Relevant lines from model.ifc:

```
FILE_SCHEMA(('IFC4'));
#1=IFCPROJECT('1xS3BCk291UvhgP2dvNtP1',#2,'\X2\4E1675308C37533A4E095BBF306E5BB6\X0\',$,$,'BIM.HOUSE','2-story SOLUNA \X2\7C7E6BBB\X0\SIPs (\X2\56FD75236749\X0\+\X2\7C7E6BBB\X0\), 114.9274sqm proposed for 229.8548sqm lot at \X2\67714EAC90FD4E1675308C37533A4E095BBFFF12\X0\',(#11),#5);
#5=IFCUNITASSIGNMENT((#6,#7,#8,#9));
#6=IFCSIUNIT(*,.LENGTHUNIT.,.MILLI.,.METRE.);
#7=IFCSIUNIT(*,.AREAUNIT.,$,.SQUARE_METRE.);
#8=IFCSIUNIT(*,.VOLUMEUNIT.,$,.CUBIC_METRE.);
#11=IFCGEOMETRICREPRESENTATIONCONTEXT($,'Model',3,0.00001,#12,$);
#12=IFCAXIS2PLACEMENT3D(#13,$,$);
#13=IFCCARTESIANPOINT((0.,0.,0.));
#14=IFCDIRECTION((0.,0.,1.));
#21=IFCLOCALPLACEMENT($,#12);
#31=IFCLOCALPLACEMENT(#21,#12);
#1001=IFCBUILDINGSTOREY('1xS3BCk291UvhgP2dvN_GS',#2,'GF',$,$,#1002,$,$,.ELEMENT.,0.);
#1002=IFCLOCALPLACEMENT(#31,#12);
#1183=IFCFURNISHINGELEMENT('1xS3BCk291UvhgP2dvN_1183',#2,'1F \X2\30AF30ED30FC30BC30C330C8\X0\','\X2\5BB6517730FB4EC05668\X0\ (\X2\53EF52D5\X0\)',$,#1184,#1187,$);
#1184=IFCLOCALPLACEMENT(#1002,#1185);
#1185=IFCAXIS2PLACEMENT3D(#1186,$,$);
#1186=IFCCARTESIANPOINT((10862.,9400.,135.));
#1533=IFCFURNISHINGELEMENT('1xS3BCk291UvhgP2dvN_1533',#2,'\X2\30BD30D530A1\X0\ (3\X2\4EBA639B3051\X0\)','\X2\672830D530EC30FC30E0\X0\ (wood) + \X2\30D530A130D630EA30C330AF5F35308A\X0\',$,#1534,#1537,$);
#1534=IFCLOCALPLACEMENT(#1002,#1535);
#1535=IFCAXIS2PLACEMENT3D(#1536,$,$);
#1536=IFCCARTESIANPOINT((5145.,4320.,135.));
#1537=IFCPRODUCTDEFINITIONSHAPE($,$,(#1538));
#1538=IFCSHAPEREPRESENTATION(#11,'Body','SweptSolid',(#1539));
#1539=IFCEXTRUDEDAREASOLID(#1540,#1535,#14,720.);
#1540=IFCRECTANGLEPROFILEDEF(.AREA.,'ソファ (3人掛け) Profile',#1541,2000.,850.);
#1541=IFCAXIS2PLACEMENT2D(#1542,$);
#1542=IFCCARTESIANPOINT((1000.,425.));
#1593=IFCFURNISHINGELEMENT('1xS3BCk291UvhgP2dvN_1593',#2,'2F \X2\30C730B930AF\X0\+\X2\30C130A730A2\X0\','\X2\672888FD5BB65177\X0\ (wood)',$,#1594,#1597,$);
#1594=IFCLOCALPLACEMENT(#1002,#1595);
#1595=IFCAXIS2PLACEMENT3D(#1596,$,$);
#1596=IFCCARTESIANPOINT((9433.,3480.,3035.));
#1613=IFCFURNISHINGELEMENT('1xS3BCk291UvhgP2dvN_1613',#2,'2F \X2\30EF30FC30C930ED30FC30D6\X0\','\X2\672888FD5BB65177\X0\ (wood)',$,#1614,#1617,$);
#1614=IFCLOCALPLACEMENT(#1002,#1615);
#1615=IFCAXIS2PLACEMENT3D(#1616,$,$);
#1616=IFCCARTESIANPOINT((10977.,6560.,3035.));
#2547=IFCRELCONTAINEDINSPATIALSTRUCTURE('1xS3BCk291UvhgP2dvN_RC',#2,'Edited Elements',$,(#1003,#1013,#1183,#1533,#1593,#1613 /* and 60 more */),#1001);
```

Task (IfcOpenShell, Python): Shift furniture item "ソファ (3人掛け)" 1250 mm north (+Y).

```python
import ifcopenshell
import ifcopenshell.api.geometry
import ifcopenshell.util.placement

model = ifcopenshell.open("model.ifc")

item = model.by_guid("1xS3BCk291UvhgP2dvN_1533")
matrix = ifcopenshell.util.placement.get_local_placement(item.ObjectPlacement)
matrix[1, 3] += 1250.0
ifcopenshell.api.geometry.edit_object_placement(model, product=item, matrix=matrix, is_si=False)

print(ifcopenshell.util.placement.get_local_placement(item.ObjectPlacement).round(3) + 0.0)

model.write("model_edited.ifc")
```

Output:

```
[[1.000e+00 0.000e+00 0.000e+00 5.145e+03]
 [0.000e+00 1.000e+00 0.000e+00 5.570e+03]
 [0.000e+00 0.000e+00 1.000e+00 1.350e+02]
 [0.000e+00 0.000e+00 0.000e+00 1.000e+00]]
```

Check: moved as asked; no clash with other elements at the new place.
